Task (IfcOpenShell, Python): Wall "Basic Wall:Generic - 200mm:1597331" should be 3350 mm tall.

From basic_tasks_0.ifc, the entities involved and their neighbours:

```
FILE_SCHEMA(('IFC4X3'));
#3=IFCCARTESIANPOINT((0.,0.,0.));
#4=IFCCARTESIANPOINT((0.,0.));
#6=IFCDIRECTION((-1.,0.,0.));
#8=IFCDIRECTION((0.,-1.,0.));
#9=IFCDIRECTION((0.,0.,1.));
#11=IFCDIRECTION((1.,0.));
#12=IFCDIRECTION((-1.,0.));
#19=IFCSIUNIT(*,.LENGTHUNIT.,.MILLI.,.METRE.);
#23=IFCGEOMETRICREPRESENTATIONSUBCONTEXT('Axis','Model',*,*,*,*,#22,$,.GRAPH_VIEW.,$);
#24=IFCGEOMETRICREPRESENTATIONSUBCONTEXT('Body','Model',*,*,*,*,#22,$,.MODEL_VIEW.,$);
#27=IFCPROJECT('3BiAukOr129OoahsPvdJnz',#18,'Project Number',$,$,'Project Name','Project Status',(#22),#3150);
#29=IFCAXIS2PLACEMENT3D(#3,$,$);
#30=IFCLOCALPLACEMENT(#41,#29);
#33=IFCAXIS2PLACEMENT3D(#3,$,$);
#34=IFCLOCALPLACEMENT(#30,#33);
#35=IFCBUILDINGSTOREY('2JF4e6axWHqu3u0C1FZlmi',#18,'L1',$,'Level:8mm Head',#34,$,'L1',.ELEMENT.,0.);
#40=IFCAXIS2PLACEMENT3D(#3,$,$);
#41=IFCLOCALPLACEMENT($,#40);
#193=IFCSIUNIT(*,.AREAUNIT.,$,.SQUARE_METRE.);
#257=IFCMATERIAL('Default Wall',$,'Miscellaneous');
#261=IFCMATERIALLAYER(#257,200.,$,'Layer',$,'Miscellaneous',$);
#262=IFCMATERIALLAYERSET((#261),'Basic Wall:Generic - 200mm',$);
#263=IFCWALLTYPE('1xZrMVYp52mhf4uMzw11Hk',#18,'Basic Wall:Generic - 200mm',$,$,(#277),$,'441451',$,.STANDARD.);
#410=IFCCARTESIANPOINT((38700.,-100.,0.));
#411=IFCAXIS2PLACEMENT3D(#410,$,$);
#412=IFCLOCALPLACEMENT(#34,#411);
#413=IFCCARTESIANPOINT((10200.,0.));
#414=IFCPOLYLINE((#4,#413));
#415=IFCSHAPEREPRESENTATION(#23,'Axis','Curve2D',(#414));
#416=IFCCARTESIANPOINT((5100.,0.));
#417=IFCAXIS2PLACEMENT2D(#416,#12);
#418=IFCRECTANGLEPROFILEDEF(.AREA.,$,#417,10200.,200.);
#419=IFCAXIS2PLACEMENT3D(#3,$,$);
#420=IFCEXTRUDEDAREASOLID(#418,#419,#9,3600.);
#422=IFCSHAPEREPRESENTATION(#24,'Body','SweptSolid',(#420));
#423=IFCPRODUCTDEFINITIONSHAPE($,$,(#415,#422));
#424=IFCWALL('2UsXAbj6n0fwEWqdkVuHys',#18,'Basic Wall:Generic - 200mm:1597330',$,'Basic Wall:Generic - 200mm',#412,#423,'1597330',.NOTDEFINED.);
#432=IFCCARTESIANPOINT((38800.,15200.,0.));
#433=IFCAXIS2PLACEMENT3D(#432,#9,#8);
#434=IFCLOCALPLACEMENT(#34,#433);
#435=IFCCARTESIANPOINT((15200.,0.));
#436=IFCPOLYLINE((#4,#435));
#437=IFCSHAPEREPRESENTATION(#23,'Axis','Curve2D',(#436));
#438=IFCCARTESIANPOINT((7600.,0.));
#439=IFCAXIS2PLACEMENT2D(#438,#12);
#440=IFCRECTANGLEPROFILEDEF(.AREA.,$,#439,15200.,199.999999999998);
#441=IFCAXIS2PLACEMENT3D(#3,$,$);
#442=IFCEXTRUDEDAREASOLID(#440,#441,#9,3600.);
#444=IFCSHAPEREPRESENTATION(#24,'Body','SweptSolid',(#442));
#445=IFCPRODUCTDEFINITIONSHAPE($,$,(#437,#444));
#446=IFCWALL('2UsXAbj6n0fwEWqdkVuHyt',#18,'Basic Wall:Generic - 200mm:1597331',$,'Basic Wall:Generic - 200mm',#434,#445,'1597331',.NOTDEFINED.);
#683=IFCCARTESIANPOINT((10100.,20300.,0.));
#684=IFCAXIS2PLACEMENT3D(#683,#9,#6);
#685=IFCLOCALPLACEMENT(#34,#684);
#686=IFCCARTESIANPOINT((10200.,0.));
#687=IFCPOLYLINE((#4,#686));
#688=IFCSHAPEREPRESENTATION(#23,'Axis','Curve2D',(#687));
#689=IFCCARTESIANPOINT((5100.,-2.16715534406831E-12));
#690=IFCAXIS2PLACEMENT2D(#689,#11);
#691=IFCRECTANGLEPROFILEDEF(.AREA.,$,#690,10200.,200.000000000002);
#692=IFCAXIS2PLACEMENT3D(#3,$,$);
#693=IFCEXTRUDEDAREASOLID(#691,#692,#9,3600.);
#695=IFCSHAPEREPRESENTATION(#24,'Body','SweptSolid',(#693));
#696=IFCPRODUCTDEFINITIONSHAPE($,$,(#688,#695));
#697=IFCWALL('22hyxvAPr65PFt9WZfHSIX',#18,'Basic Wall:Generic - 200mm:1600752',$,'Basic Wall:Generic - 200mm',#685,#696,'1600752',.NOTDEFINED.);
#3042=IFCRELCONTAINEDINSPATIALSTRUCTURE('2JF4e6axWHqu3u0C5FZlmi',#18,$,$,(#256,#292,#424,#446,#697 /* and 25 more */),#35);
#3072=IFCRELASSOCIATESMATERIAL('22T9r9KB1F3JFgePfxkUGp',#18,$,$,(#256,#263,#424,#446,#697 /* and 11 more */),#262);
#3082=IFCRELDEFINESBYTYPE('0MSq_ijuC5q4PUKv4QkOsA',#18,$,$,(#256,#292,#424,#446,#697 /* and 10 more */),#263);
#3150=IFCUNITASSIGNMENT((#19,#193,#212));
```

```python
import ifcopenshell
import ifcopenshell.geom
import ifcopenshell.util.representation
import ifcopenshell.util.shape
import ifcopenshell.util.unit

model = ifcopenshell.open("basic_tasks_0.ifc")
unit_scale = ifcopenshell.util.unit.calculate_unit_scale(model)
settings = ifcopenshell.geom.settings()


def volume(element):
    """Net volume in cubic metres, openings subtracted."""
    shape = ifcopenshell.geom.create_shape(settings, element)
    return ifcopenshell.util.shape.get_volume(shape.geometry)


wall = model.by_guid("2UsXAbj6n0fwEWqdkVuHyt")
before = volume(wall)

body = ifcopenshell.util.representation.get_representation(wall, "Model", "Body")
solid = body.Items[0]
old_height = solid.Depth
solid.Depth = 3.35 / unit_scale
after = volume(wall)

print(f"height {old_height:g} -> {solid.Depth:g}, volume {before:.3f} -> {after:.3f} m3")

model.write("basic_tasks_0-out.ifc")
```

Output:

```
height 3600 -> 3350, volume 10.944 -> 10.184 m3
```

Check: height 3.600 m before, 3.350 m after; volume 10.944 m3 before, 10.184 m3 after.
